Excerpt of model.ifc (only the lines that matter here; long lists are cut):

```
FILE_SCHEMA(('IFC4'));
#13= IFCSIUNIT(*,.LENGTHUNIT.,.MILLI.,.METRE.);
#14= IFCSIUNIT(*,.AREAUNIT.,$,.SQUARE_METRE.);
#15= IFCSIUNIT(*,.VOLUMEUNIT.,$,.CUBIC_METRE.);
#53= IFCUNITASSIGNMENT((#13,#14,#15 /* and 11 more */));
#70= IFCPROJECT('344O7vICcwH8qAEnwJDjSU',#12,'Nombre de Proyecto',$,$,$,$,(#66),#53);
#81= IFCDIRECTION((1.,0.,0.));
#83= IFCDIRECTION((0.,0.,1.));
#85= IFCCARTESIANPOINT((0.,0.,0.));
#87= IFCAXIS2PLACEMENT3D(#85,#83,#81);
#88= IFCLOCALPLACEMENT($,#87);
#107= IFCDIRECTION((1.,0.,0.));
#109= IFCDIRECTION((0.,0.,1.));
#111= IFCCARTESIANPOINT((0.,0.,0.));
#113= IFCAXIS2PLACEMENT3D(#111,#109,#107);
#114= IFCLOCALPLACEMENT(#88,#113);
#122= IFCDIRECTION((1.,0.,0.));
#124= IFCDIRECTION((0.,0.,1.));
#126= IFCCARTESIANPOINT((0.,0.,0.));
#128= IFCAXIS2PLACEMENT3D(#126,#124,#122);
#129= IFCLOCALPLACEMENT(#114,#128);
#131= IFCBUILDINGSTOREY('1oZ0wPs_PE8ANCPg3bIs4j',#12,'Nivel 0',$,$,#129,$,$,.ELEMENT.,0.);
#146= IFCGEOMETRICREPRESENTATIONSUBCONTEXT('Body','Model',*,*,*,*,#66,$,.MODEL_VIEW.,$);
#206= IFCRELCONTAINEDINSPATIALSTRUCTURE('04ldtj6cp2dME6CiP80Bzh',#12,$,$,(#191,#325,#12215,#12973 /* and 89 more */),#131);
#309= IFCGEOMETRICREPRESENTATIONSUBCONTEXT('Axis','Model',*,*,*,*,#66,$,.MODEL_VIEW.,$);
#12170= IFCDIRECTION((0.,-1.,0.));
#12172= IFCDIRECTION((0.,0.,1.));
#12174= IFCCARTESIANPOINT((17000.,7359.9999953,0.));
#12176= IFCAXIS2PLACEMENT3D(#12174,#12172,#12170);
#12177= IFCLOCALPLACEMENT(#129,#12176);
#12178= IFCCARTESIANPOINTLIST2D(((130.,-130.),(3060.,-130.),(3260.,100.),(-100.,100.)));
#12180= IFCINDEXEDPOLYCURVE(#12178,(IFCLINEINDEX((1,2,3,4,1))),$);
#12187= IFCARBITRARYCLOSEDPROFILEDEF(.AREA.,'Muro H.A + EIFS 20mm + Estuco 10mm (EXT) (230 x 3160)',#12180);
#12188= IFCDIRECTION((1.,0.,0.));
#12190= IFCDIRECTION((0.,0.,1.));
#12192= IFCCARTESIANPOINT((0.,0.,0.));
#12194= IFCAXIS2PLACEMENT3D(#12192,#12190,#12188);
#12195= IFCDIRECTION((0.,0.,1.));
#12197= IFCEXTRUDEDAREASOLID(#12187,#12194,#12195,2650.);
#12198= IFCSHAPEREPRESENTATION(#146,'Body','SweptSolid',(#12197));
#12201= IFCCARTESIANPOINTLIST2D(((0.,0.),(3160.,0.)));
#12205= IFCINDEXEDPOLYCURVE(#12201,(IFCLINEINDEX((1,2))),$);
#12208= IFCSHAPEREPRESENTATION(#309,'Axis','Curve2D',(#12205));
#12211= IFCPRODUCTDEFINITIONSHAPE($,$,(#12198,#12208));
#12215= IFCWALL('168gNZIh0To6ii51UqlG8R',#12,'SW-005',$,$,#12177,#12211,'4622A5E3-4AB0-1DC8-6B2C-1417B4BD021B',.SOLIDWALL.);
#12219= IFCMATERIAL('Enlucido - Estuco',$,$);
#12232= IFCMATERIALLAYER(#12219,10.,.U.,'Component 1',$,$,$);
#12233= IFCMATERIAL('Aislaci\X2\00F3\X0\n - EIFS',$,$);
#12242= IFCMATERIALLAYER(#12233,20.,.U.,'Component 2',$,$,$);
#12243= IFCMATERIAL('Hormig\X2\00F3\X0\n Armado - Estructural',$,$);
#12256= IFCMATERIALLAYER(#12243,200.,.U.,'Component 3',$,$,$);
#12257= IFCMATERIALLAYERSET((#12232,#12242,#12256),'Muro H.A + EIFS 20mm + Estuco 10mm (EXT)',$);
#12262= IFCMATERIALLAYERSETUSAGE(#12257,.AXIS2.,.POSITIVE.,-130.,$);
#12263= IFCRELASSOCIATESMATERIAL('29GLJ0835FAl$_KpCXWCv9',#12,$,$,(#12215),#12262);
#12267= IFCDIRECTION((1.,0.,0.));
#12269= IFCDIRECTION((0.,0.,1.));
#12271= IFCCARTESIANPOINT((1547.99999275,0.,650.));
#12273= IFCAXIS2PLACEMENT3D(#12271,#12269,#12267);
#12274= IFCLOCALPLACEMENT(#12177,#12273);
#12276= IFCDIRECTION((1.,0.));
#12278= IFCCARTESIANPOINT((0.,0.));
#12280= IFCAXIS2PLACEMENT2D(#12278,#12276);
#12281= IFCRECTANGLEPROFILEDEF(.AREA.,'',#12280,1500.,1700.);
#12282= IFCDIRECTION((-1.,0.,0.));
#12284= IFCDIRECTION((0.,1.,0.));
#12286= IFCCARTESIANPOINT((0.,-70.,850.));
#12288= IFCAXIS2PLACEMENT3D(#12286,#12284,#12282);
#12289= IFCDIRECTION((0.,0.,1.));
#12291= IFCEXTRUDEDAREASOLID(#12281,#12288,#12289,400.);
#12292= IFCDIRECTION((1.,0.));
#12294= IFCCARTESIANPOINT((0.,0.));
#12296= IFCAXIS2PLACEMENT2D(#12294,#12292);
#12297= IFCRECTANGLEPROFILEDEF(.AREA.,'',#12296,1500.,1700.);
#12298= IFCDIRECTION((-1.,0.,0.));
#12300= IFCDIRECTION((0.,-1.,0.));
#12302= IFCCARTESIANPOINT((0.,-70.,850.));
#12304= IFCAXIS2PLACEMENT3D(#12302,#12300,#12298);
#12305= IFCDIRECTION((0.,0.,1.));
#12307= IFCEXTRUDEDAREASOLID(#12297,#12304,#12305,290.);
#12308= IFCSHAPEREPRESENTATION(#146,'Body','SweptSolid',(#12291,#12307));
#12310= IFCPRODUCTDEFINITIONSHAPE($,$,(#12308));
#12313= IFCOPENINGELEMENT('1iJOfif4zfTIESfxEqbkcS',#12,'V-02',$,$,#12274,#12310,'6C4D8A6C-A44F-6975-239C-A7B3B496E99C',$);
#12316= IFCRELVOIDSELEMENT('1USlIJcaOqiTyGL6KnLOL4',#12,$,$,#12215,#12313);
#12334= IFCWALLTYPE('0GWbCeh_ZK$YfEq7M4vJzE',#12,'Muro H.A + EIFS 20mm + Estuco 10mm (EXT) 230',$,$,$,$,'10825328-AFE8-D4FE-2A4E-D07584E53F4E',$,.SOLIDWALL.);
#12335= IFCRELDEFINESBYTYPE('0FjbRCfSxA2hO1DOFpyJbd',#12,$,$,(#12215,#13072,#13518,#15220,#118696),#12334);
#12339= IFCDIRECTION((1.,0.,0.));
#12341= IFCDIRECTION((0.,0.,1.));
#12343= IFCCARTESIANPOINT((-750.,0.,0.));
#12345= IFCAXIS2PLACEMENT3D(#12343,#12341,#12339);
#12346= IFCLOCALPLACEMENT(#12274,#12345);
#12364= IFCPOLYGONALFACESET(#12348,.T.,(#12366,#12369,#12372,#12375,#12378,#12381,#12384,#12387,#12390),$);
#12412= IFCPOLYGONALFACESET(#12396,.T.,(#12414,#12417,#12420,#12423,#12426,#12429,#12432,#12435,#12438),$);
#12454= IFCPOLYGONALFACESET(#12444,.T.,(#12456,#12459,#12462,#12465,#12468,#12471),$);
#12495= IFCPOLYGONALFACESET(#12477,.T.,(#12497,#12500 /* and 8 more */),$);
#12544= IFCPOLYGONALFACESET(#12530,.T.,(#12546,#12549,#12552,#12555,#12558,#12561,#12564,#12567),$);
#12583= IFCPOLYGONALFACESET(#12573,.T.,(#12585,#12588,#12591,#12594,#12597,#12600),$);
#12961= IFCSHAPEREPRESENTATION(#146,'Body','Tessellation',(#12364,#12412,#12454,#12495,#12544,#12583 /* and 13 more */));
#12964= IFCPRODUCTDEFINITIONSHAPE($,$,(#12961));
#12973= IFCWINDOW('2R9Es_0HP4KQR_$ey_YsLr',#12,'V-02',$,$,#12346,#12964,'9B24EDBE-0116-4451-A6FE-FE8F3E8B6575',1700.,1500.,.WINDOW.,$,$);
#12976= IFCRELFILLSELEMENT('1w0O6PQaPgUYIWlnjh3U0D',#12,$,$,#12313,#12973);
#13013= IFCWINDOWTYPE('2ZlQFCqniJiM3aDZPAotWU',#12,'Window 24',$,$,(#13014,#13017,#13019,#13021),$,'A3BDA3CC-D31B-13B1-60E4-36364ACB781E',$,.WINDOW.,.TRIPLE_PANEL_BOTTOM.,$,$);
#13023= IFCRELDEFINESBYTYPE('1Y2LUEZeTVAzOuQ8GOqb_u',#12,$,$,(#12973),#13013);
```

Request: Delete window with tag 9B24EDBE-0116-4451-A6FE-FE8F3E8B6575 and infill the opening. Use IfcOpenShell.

```python
import ifcopenshell
import ifcopenshell.api.feature
import ifcopenshell.api.root
import ifcopenshell.geom
import ifcopenshell.util.shape

model = ifcopenshell.open("model.ifc")
settings = ifcopenshell.geom.settings()


def volume(element):
    """Net volume in cubic metres, openings subtracted."""
    shape = ifcopenshell.geom.create_shape(settings, element)
    return ifcopenshell.util.shape.get_volume(shape.geometry)


window = model.by_guid("2R9Es_0HP4KQR_$ey_YsLr")
opening = window.FillsVoids[0].RelatingOpeningElement
wall = opening.VoidsElements[0].RelatingBuildingElement
before = volume(wall)

ifcopenshell.api.root.remove_product(model, product=window)
ifcopenshell.api.feature.remove_feature(model, feature=opening)

after = volume(wall)

print(f"wall volume {before:.3f} -> {after:.3f} m3")

model.write("model_edited.ifc")
```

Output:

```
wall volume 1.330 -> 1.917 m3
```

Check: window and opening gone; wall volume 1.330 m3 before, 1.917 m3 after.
